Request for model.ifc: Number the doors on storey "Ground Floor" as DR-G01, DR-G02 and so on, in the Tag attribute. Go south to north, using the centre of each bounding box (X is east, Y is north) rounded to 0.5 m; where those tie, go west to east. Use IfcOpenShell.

First a look at what the model holds.

```python
import ifcopenshell
import ifcopenshell.util.element
import ifcopenshell.util.placement

model = ifcopenshell.open("model.ifc")
print(model.schema)
storey = next(s for s in model.by_type("IfcBuildingStorey") if s.Name == "Ground Floor")
doors = [e for e in ifcopenshell.util.element.get_decomposition(storey) if e.is_a("IfcDoor")]
for e in sorted(doors, key=lambda e: e.id()):
    origin = ifcopenshell.util.placement.get_local_placement(e.ObjectPlacement)[:3, 3]
    print(e.id(), e.Tag, e.Name, origin.round(2) + 0.0, sep=" | ")
```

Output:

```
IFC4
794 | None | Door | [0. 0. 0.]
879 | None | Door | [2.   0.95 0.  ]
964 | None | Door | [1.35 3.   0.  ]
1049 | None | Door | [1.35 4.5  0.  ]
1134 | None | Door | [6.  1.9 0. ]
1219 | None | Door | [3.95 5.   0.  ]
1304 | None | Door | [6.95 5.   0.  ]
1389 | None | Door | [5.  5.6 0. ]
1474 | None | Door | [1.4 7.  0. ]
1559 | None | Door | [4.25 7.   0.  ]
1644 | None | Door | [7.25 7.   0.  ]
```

```python
import ifcopenshell
import ifcopenshell.geom
import ifcopenshell.util.element
import ifcopenshell.util.shape

model = ifcopenshell.open("model.ifc")
settings = ifcopenshell.geom.settings()
settings.set("use-world-coords", True)


def centre(element):
    shape = ifcopenshell.geom.create_shape(settings, element)
    return ifcopenshell.util.shape.get_bbox_centroid(shape.geometry)


storey = next(s for s in model.by_type("IfcBuildingStorey") if s.Name == "Ground Floor")
doors = [e for e in ifcopenshell.util.element.get_decomposition(storey) if e.is_a("IfcDoor")]

# Insertion points can sit at a corner or the storey origin, so sort by the geometry (in metres).
centres = {e: centre(e) for e in doors}
doors.sort(key=lambda e: (round(centres[e][1] / 0.5), centres[e][0]))

for i, e in enumerate(doors, start=1):
    number = f"DR-G{i:02d}"
    e.Tag = number
    print(e.id(), number)

model.write("model_rev.ifc")
```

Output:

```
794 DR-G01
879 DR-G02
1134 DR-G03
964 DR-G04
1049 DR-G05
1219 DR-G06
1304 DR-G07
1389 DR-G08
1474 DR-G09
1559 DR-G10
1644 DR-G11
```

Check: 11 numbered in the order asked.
